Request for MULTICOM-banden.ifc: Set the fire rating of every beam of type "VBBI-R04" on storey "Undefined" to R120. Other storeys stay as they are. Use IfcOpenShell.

First a look at what the model holds.

```python
import ifcopenshell
import ifcopenshell.util.element

model = ifcopenshell.open("MULTICOM-banden.ifc")
print(model.schema)
storey = next(s for s in model.by_type("IfcBuildingStorey") if s.Name == "Undefined")
beams = [e for e in ifcopenshell.util.element.get_decomposition(storey) if e.is_a("IfcBeam")]
seen = {}
for e in beams:
    element_type = ifcopenshell.util.element.get_type(e)
    key = (element_type.Name if element_type != e and element_type else None, ifcopenshell.util.element.get_pset(e, "Pset_BeamCommon", "FireRating"))
    seen[key] = seen.get(key, 0) + 1
for (name, value), count in sorted(seen.items(), key=str):
    print(count, "x", name, "|", value)
```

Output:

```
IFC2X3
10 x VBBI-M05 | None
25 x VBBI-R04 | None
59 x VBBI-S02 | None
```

```python
import ifcopenshell
import ifcopenshell.api.pset
import ifcopenshell.util.element

model = ifcopenshell.open("MULTICOM-banden.ifc")

storey = next(s for s in model.by_type("IfcBuildingStorey") if s.Name == "Undefined")
beams = [e for e in ifcopenshell.util.element.get_decomposition(storey) if e.is_a("IfcBeam")]

count = 0
for e in beams:
    element_type = ifcopenshell.util.element.get_type(e)
    if element_type in (None, e) or element_type.Name != "VBBI-R04":
        continue
    # add_pset returns the element's existing set when there is one.
    pset = ifcopenshell.api.pset.add_pset(model, product=e, name="Pset_BeamCommon")
    ifcopenshell.api.pset.edit_pset(model, pset=pset, properties={"FireRating": "R120"})
    count += 1

print(count, "beams updated")

model.write("MULTICOM-banden_rev.ifc")
```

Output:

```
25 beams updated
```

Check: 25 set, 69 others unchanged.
